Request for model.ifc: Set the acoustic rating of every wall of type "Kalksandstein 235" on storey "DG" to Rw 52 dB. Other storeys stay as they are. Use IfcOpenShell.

First a look at what the model holds.

```python
import ifcopenshell
import ifcopenshell.util.element

model = ifcopenshell.open("model.ifc")
print(model.schema)
storey = next(s for s in model.by_type("IfcBuildingStorey") if s.Name == "DG")
walls = [e for e in ifcopenshell.util.element.get_decomposition(storey) if e.is_a("IfcWall")]
seen = {}
for e in walls:
    element_type = ifcopenshell.util.element.get_type(e)
    key = (element_type.Name if element_type != e and element_type else None, ifcopenshell.util.element.get_pset(e, "Pset_WallCommon", "AcousticRating"))
    seen[key] = seen.get(key, 0) + 1
for (name, value), count in sorted(seen.items(), key=str):
    print(count, "x", name, "|", value)
```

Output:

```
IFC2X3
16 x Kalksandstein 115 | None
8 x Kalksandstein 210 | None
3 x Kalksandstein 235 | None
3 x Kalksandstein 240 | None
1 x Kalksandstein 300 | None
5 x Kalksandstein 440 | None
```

```python
import ifcopenshell
import ifcopenshell.api.pset
import ifcopenshell.util.element

model = ifcopenshell.open("model.ifc")

storey = next(s for s in model.by_type("IfcBuildingStorey") if s.Name == "DG")
walls = [e for e in ifcopenshell.util.element.get_decomposition(storey) if e.is_a("IfcWall")]

count = 0
for e in walls:
    element_type = ifcopenshell.util.element.get_type(e)
    if element_type in (None, e) or element_type.Name != "Kalksandstein 235":
        continue
    # add_pset returns the element's existing set when there is one.
    pset = ifcopenshell.api.pset.add_pset(model, product=e, name="Pset_WallCommon")
    ifcopenshell.api.pset.edit_pset(model, pset=pset, properties={"AcousticRating": "Rw 52 dB"})
    count += 1

print(count, "walls updated")

model.write("model_rev.ifc")
```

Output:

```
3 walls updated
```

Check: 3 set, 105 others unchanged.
